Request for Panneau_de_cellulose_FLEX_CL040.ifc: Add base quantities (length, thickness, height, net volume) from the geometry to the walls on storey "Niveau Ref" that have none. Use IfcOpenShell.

First a look at what the model holds.

```python
import ifcopenshell
import ifcopenshell.util.element
import ifcopenshell.util.unit

model = ifcopenshell.open("Panneau_de_cellulose_FLEX_CL040.ifc")
print(model.schema)
for unit_type in ("LENGTHUNIT", "AREAUNIT", "VOLUMEUNIT"):
    print(unit_type, ifcopenshell.util.unit.calculate_unit_scale(model, unit_type))
storey = next(s for s in model.by_type("IfcBuildingStorey") if s.Name == "Niveau Ref")
walls = [e for e in ifcopenshell.util.element.get_decomposition(storey) if e.is_a("IfcWall")]
for e in sorted(walls, key=lambda e: e.id()):
    print(e.id(), e.is_a(), e.Name, list(ifcopenshell.util.element.get_psets(e, qtos_only=True)), sep=" | ")
```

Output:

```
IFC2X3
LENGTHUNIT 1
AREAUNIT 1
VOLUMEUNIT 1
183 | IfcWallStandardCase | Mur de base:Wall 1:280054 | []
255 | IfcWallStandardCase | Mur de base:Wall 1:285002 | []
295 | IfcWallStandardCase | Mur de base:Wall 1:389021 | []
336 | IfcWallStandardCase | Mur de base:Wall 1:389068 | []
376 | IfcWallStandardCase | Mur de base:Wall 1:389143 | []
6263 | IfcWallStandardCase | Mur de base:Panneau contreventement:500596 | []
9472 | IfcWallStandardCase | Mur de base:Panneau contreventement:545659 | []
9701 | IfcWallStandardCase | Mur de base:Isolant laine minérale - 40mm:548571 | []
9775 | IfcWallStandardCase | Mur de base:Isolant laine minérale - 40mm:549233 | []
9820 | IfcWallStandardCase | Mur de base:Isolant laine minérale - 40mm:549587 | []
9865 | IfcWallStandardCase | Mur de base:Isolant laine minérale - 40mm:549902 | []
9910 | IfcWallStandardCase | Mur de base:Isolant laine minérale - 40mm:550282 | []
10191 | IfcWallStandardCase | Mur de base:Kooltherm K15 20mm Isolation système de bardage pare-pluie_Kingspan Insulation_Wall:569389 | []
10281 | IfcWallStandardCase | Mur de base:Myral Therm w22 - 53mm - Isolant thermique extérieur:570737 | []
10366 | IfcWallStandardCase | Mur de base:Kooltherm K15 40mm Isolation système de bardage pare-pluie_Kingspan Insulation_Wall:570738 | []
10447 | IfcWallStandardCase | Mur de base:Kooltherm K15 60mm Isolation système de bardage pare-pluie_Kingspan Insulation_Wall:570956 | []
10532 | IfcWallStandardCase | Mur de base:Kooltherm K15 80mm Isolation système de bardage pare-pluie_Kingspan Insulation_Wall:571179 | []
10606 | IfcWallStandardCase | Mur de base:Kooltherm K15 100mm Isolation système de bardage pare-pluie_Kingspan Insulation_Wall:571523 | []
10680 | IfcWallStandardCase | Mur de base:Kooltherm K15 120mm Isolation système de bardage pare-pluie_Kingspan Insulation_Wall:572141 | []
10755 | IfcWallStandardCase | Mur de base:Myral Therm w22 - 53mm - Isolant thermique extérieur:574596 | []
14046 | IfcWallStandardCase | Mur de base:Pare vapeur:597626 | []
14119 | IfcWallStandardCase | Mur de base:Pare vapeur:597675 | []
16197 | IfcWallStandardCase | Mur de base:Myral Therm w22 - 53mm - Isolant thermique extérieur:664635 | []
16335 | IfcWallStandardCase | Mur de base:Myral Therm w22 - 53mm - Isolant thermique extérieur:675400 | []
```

```python
import ifcopenshell
import ifcopenshell.api.pset
import ifcopenshell.geom
import ifcopenshell.util.element
import ifcopenshell.util.shape
import ifcopenshell.util.unit

model = ifcopenshell.open("Panneau_de_cellulose_FLEX_CL040.ifc")
unit_scale = ifcopenshell.util.unit.calculate_unit_scale(model)
volume_scale = ifcopenshell.util.unit.calculate_unit_scale(model, "VOLUMEUNIT")
settings = ifcopenshell.geom.settings()

storey = next(s for s in model.by_type("IfcBuildingStorey") if s.Name == "Niveau Ref")
walls = [e for e in ifcopenshell.util.element.get_decomposition(storey) if e.is_a("IfcWall")]

for e in sorted(walls, key=lambda e: e.id()):
    if ifcopenshell.util.element.get_psets(e, qtos_only=True, should_inherit=False):
        continue
    # Geometry comes back in metres, in the element's own axes.
    shape = ifcopenshell.geom.create_shape(settings, e)
    values = {
        "Length": ifcopenshell.util.shape.get_x(shape.geometry) / unit_scale,
        "Width": ifcopenshell.util.shape.get_y(shape.geometry) / unit_scale,
        "Height": ifcopenshell.util.shape.get_z(shape.geometry) / unit_scale,
        "NetVolume": ifcopenshell.util.shape.get_volume(shape.geometry) / volume_scale,
    }
    qto = ifcopenshell.api.pset.add_qto(model, product=e, name="BaseQuantities")
    ifcopenshell.api.pset.edit_qto(model, qto=qto, properties=values)
    print(e.id(), {k: round(v, 3) for k, v in values.items()})

model.write("Panneau_de_cellulose_FLEX_CL040_updated.ifc")
```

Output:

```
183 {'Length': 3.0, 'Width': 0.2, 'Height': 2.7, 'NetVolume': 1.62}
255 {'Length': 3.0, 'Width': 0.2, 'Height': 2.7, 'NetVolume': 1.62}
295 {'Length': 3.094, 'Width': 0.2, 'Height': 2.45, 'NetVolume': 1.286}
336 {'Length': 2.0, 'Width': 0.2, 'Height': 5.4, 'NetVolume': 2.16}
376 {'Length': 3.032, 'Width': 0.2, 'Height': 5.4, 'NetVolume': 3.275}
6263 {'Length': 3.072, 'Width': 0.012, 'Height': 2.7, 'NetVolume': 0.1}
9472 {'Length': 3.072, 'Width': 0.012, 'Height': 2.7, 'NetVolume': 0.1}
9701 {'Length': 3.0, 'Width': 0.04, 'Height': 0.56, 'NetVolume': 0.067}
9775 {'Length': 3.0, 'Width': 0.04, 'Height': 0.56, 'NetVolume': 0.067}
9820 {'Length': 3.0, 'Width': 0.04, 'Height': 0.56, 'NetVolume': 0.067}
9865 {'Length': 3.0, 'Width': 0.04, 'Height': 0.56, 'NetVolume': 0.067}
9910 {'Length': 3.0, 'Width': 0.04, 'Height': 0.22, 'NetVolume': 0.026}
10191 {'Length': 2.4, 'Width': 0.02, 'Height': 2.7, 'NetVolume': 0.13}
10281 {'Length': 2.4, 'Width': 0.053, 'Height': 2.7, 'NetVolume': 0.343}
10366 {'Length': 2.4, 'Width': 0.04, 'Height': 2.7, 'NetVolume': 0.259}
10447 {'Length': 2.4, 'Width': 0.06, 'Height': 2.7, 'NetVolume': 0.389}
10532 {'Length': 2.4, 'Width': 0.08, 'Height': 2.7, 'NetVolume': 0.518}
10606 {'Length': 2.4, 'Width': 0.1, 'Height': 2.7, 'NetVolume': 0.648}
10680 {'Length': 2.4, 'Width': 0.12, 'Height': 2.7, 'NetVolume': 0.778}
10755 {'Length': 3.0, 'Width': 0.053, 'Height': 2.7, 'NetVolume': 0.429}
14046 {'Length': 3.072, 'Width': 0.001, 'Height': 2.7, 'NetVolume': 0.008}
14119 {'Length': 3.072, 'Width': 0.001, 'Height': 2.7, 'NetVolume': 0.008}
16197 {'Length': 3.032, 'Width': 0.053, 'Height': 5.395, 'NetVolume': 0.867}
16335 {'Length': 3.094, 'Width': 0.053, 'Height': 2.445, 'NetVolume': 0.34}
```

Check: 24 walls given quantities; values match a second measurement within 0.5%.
